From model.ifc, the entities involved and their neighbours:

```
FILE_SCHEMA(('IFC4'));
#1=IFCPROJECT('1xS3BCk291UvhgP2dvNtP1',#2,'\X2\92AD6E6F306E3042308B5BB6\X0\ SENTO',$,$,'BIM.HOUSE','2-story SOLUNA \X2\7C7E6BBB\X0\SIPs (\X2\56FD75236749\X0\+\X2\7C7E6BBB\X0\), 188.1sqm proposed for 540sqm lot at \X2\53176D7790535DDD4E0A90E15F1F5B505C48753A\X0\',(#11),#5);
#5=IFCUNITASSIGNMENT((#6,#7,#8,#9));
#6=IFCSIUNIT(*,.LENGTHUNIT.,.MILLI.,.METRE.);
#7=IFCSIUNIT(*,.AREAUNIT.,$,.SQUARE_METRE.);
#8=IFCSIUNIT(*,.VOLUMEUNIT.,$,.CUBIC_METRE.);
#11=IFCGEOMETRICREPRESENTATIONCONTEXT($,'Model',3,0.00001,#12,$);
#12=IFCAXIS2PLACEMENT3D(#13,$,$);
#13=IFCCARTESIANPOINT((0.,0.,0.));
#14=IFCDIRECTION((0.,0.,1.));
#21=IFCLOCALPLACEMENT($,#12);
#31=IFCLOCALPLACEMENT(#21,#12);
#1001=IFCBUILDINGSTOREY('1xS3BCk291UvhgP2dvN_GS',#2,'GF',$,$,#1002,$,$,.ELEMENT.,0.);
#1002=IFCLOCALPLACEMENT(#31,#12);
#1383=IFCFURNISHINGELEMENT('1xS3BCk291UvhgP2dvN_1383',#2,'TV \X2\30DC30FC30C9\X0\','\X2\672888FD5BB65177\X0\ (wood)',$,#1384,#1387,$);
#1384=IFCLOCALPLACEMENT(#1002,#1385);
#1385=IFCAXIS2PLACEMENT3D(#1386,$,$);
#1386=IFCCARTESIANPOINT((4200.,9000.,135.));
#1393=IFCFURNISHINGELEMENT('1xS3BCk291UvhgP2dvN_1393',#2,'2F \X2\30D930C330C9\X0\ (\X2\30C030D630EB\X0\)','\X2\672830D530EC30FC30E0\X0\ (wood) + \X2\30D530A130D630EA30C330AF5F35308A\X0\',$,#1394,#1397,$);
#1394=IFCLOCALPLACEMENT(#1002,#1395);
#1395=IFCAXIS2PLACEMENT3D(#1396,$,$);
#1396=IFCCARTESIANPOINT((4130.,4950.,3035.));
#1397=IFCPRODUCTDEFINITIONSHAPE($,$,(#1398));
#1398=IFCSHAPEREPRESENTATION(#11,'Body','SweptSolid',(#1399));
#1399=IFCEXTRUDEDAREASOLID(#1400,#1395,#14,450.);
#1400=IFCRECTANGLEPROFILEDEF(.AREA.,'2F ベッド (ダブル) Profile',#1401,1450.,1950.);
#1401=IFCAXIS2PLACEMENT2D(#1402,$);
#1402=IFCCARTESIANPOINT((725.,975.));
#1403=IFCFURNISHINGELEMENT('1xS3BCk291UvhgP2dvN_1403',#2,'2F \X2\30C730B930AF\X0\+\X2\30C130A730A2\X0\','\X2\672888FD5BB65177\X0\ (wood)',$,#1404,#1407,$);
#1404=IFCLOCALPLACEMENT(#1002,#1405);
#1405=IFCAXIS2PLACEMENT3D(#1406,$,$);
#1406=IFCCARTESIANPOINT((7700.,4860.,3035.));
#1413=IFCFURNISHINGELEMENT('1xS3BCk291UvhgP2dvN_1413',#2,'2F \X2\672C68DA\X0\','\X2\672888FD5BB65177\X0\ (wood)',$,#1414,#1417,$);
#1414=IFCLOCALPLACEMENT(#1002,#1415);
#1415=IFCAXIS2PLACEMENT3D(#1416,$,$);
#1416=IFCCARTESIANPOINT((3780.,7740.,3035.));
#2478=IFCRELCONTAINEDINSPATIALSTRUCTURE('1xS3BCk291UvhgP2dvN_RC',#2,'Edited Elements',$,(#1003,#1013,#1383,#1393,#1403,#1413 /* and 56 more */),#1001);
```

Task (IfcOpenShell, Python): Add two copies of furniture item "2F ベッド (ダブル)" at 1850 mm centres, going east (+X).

```python
import numpy as np
import ifcopenshell
import ifcopenshell.api.geometry
import ifcopenshell.api.root
import ifcopenshell.util.element
import ifcopenshell.util.placement
import ifcopenshell.util.unit

model = ifcopenshell.open("model.ifc")
unit_scale = ifcopenshell.util.unit.calculate_unit_scale(model)


def reuse_history(source, copy):
    """copy_class also copies each property set's owner history, people and application; keep the originals."""
    for rel in copy.IsDefinedBy:
        if rel.is_a("IfcRelDefinesByProperties") and (history := rel.RelatingPropertyDefinition.OwnerHistory):
            rel.RelatingPropertyDefinition.OwnerHistory = source.OwnerHistory
            ifcopenshell.util.element.remove_deep2(model, history)


source = model.by_id(1393)
base = ifcopenshell.util.placement.get_local_placement(source.ObjectPlacement)
step = np.array([1.0, 0.0, 0.0]) * 1.85 / unit_scale

for i in range(1, 3):
    copy = ifcopenshell.api.root.copy_class(model, product=source)
    copy.Representation = ifcopenshell.util.element.copy_deep(
        model, source.Representation, exclude=["IfcGeometricRepresentationContext", "IfcRepresentationMap"]
    )
    reuse_history(source, copy)
    matrix = base.copy()
    matrix[:3, 3] += i * step
    print("added at", matrix[:3, 3].round(3) + 0.0)
    ifcopenshell.api.geometry.edit_object_placement(model, product=copy, matrix=matrix, is_si=False)

model.write("model_edited.ifc")
```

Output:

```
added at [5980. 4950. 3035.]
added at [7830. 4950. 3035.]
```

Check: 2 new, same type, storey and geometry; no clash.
